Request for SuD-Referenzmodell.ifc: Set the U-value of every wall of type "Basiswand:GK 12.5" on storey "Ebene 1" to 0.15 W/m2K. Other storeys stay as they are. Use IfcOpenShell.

First a look at what the model holds.

```python
import ifcopenshell
import ifcopenshell.util.element

model = ifcopenshell.open("SuD-Referenzmodell.ifc")
print(model.schema)
storey = next(s for s in model.by_type("IfcBuildingStorey") if s.Name == "Ebene 1")
walls = [e for e in ifcopenshell.util.element.get_decomposition(storey) if e.is_a("IfcWall")]
seen = {}
for e in walls:
    element_type = ifcopenshell.util.element.get_type(e)
    key = (element_type.Name if element_type != e and element_type else None, ifcopenshell.util.element.get_pset(e, "Pset_WallCommon", "ThermalTransmittance"))
    seen[key] = seen.get(key, 0) + 1
for (name, value), count in sorted(seen.items(), key=str):
    print(count, "x", name, "|", value)
```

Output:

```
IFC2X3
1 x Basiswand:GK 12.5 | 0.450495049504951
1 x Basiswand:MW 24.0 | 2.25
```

```python
import ifcopenshell
import ifcopenshell.api.pset
import ifcopenshell.util.element

model = ifcopenshell.open("SuD-Referenzmodell.ifc")

storey = next(s for s in model.by_type("IfcBuildingStorey") if s.Name == "Ebene 1")
walls = [e for e in ifcopenshell.util.element.get_decomposition(storey) if e.is_a("IfcWall")]

count = 0
for e in walls:
    element_type = ifcopenshell.util.element.get_type(e)
    if element_type in (None, e) or element_type.Name != "Basiswand:GK 12.5":
        continue
    # add_pset returns the element's existing set when there is one.
    pset = ifcopenshell.api.pset.add_pset(model, product=e, name="Pset_WallCommon")
    ifcopenshell.api.pset.edit_pset(model, pset=pset, properties={"ThermalTransmittance": 0.15})
    count += 1

print(count, "walls updated")

model.write("SuD-Referenzmodell_edited.ifc")
```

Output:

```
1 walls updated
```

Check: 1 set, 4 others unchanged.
